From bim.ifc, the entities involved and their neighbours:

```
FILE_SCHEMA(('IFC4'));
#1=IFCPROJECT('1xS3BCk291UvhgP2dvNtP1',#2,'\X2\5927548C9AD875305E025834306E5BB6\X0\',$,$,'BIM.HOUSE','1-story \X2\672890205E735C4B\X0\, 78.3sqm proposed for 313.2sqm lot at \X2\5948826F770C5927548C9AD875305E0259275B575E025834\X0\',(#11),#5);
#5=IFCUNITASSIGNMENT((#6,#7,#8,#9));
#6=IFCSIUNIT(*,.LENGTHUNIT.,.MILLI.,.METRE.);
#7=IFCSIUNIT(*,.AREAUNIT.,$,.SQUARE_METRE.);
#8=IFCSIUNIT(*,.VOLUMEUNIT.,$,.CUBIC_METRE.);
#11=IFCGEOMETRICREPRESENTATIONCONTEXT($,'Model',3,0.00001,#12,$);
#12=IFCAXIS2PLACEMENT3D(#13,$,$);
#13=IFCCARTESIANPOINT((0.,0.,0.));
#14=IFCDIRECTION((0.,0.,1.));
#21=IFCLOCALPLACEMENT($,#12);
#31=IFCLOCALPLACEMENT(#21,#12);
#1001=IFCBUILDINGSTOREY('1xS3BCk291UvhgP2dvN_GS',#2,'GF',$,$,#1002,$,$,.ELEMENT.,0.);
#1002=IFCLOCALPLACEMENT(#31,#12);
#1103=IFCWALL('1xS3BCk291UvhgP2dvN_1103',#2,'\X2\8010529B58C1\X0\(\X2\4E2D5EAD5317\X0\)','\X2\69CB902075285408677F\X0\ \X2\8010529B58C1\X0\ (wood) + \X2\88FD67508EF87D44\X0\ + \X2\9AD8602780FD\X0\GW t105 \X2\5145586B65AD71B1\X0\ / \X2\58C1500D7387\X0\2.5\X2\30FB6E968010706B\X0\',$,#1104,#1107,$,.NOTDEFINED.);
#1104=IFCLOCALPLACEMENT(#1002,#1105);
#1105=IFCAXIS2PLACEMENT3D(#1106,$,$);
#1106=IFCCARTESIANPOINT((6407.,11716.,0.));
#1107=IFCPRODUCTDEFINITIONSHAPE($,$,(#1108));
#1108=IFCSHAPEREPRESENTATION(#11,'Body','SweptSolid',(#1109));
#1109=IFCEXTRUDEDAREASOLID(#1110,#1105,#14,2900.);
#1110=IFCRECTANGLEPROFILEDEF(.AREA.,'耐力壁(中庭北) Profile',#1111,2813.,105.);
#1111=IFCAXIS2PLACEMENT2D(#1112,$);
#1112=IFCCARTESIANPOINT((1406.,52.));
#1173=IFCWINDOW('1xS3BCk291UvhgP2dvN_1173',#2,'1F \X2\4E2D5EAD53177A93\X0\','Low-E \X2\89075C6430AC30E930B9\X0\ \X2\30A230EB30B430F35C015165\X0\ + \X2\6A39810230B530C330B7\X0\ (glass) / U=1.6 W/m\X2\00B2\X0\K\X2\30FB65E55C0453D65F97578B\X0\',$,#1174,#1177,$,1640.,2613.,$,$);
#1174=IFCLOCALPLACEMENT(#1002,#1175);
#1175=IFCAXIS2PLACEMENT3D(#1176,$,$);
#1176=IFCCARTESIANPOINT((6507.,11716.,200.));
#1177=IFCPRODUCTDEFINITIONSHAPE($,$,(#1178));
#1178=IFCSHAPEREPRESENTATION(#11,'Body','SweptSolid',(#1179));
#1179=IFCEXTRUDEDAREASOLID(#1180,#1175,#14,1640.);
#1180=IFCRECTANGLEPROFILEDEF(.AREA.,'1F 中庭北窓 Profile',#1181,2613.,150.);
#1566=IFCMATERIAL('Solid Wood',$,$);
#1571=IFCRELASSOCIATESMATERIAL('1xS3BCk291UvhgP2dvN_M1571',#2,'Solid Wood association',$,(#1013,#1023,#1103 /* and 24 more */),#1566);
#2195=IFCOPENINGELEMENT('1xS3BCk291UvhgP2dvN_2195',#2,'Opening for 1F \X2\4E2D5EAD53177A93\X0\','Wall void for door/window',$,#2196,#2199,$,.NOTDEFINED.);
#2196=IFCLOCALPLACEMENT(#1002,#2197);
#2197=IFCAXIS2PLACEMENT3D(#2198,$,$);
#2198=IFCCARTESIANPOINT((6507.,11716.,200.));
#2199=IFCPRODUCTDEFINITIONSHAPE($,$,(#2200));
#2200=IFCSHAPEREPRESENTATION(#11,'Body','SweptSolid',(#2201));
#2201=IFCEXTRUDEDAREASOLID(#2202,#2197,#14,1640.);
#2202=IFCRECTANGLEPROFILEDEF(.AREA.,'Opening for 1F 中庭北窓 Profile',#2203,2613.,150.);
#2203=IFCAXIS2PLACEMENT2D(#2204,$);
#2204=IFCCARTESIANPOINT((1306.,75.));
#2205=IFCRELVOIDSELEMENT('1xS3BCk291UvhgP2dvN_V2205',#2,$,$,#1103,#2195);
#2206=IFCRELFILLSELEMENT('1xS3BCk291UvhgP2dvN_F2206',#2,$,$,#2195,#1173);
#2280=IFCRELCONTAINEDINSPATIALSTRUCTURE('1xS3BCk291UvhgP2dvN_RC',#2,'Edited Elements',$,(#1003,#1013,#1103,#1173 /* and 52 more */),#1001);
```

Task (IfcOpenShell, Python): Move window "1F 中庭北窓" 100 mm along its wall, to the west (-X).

```python
import ifcopenshell
import ifcopenshell.api.geometry
import ifcopenshell.util.placement

model = ifcopenshell.open("bim.ifc")

window = model.by_guid("1xS3BCk291UvhgP2dvN_1173")
opening = window.FillsVoids[0].RelatingOpeningElement
wall = opening.VoidsElements[0].RelatingBuildingElement

wall_matrix = ifcopenshell.util.placement.get_local_placement(wall.ObjectPlacement)
shift = wall_matrix[:3, 0] * -100.0
before = ifcopenshell.util.placement.get_local_placement(window.ObjectPlacement)[:3, 3].copy()

# The window is not placed relative to its opening, so move both.
for product in (opening, window):
    matrix = ifcopenshell.util.placement.get_local_placement(product.ObjectPlacement)
    matrix[:3, 3] += shift
    ifcopenshell.api.geometry.edit_object_placement(model, product=product, matrix=matrix, is_si=False)

after = ifcopenshell.util.placement.get_local_placement(window.ObjectPlacement)[:3, 3]
print("window moved by", (after - before).round(3) + 0.0)

model.write("bim_edited.ifc")
```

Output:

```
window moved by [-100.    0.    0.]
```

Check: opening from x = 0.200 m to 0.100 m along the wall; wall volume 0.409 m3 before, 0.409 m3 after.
